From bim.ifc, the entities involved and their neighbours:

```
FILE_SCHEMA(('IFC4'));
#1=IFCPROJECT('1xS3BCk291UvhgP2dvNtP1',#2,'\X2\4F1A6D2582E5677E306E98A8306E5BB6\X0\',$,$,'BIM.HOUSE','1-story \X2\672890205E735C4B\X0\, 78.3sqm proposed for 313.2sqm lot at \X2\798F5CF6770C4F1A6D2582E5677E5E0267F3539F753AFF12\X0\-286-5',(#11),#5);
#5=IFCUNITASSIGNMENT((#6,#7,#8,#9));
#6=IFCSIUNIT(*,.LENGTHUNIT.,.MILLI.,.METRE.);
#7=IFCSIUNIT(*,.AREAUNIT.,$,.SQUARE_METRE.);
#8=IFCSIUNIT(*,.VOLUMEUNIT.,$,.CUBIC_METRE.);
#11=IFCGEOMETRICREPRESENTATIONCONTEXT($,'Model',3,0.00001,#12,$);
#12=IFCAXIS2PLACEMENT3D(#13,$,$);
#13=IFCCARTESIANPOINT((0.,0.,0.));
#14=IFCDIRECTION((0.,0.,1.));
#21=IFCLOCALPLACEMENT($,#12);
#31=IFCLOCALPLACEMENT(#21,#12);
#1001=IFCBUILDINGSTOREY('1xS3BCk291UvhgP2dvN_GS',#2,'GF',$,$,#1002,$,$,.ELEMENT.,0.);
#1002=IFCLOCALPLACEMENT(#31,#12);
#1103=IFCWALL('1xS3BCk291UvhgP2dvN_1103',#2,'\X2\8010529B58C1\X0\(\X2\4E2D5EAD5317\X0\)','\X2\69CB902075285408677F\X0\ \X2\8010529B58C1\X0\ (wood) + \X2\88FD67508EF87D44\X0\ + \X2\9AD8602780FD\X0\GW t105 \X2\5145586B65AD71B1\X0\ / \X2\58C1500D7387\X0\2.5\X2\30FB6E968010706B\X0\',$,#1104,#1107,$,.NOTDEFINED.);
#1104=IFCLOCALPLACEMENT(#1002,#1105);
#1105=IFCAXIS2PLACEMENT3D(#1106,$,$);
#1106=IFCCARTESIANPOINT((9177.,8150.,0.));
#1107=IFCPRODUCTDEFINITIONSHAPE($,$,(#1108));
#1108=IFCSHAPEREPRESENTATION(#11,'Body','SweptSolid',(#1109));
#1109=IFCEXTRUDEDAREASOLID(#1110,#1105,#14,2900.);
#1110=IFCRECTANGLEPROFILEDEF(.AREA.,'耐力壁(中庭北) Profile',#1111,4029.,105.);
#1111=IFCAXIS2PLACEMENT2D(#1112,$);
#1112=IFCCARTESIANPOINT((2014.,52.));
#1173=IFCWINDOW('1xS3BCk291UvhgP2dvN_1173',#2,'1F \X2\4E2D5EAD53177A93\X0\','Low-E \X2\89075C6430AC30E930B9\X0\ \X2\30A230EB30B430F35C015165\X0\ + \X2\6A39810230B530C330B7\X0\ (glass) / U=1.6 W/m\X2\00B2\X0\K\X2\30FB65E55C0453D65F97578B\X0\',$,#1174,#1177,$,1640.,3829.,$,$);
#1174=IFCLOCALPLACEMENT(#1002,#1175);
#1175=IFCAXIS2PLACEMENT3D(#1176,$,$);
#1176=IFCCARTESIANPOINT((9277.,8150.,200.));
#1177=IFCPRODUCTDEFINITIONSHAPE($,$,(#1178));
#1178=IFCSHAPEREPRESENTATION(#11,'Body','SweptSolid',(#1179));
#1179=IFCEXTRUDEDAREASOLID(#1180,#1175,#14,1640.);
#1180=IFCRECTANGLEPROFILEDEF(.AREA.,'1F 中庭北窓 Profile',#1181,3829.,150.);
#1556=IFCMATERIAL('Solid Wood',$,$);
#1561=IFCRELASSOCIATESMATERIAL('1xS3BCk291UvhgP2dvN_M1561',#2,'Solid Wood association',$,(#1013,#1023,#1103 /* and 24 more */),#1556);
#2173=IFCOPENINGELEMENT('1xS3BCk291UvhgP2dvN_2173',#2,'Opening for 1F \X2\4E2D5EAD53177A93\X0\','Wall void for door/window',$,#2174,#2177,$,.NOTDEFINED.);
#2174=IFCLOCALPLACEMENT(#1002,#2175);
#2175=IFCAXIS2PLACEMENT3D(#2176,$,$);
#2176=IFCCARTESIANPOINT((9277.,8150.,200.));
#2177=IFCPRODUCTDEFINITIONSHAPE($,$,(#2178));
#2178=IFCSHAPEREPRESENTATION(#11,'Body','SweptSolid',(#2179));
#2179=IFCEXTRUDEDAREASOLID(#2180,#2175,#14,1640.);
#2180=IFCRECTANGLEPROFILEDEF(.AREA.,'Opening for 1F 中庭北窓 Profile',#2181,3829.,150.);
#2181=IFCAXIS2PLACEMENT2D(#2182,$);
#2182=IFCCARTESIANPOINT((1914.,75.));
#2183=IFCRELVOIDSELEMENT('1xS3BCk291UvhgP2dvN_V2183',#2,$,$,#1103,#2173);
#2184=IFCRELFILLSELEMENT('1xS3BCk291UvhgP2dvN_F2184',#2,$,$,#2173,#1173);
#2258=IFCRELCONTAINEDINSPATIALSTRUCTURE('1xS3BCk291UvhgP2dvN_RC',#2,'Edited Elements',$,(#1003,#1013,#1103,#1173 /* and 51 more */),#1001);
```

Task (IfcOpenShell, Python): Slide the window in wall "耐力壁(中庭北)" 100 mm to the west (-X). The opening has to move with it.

```python
import ifcopenshell
import ifcopenshell.api.geometry
import ifcopenshell.util.placement

model = ifcopenshell.open("bim.ifc")

window = model.by_guid("1xS3BCk291UvhgP2dvN_1173")
opening = window.FillsVoids[0].RelatingOpeningElement
wall = opening.VoidsElements[0].RelatingBuildingElement

wall_matrix = ifcopenshell.util.placement.get_local_placement(wall.ObjectPlacement)
shift = wall_matrix[:3, 0] * -100.0
before = ifcopenshell.util.placement.get_local_placement(window.ObjectPlacement)[:3, 3].copy()

# The window is not placed relative to its opening, so move both.
for product in (opening, window):
    matrix = ifcopenshell.util.placement.get_local_placement(product.ObjectPlacement)
    matrix[:3, 3] += shift
    ifcopenshell.api.geometry.edit_object_placement(model, product=product, matrix=matrix, is_si=False)

after = ifcopenshell.util.placement.get_local_placement(window.ObjectPlacement)[:3, 3]
print("window moved by", (after - before).round(3) + 0.0)

model.write("bim_updated.ifc")
```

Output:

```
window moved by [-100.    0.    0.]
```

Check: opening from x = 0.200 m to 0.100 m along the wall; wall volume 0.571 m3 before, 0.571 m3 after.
